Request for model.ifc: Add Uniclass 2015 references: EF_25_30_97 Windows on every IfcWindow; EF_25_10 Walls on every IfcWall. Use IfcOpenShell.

First a look at what the model holds.

```python
import ifcopenshell

model = ifcopenshell.open("model.ifc")
print(model.schema)
print("classifications:", [c.Name for c in model.by_type("IfcClassification")])
for ifc_class in ("IfcDoor", "IfcRoof", "IfcStair", "IfcWall", "IfcWindow"):
    print(ifc_class, len(model.by_type(ifc_class)))
```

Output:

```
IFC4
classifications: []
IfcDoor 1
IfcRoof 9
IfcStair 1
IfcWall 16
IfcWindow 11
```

```python
import ifcopenshell
import ifcopenshell.api.classification

model = ifcopenshell.open("model.ifc")

system = ifcopenshell.api.classification.add_classification(model, classification="Uniclass 2015")

codes = {
    "IfcWindow": ("EF_25_30_97", "Windows"),
    "IfcWall": ("EF_25_10", "Walls"),
}
for ifc_class, (code, name) in codes.items():
    products = model.by_type(ifc_class)
    ifcopenshell.api.classification.add_reference(
        model, products=products, classification=system, identification=code, name=name
    )
    print(code, len(products))

model.write("model_updated.ifc")
```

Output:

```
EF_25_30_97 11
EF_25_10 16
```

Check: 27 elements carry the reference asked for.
